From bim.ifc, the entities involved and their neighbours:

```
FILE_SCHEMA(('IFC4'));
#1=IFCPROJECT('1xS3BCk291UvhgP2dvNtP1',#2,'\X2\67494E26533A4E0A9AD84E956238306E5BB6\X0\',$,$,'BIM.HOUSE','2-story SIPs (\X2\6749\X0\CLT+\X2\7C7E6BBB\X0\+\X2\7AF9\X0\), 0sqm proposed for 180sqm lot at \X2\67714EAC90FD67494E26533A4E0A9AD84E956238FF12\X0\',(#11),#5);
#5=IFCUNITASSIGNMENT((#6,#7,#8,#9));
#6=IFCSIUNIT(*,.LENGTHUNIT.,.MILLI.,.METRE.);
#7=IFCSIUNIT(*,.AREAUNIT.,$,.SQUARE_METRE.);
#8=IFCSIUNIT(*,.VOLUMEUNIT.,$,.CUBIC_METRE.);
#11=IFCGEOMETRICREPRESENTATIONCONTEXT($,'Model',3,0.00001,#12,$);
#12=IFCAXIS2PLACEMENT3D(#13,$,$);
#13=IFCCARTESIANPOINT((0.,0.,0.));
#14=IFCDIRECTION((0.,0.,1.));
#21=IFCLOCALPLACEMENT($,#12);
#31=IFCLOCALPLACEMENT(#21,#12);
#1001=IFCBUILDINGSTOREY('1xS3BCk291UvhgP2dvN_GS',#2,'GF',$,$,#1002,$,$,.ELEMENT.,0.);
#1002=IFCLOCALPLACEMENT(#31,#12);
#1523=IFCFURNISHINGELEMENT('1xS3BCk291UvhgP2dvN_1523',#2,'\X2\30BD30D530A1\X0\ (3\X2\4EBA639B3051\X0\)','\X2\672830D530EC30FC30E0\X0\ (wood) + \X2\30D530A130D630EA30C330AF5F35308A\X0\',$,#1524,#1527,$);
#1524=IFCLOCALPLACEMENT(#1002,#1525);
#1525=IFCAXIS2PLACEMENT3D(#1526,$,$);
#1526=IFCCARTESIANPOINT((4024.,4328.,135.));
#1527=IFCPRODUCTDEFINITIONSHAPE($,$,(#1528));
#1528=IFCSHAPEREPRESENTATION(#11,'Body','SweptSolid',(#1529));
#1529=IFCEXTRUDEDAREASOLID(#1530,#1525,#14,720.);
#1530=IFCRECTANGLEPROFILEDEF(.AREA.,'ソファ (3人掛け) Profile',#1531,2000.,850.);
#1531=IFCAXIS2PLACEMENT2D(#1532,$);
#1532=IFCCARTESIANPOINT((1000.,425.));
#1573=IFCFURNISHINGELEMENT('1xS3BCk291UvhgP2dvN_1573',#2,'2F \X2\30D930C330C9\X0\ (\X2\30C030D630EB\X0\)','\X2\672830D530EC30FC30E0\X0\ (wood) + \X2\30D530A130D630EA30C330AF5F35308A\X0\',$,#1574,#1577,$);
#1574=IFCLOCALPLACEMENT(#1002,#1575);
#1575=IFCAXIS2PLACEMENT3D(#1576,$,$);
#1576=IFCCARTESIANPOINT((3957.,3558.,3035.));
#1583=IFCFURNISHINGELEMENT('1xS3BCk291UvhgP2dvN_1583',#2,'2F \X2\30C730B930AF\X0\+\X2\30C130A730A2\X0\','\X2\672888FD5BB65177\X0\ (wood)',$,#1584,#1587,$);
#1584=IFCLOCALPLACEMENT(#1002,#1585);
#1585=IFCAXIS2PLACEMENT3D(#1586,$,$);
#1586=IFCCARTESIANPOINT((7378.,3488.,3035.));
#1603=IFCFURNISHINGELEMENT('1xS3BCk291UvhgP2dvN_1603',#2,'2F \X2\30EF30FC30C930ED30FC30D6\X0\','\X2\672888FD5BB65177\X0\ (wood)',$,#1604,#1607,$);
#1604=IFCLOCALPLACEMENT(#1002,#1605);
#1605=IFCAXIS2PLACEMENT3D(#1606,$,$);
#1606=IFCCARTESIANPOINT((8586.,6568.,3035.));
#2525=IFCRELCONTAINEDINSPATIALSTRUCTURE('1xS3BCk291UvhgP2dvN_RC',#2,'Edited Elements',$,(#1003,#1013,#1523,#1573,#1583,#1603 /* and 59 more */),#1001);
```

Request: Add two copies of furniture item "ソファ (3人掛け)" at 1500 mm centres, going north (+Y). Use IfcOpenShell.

```python
import numpy as np
import ifcopenshell
import ifcopenshell.api.geometry
import ifcopenshell.api.root
import ifcopenshell.util.element
import ifcopenshell.util.placement
import ifcopenshell.util.unit

model = ifcopenshell.open("bim.ifc")
unit_scale = ifcopenshell.util.unit.calculate_unit_scale(model)


def reuse_history(source, copy):
    """copy_class also copies each property set's owner history, people and application; keep the originals."""
    for rel in copy.IsDefinedBy:
        if rel.is_a("IfcRelDefinesByProperties") and (history := rel.RelatingPropertyDefinition.OwnerHistory):
            rel.RelatingPropertyDefinition.OwnerHistory = source.OwnerHistory
            ifcopenshell.util.element.remove_deep2(model, history)


source = model.by_guid("1xS3BCk291UvhgP2dvN_1523")
base = ifcopenshell.util.placement.get_local_placement(source.ObjectPlacement)
step = np.array([0.0, 1.0, 0.0]) * 1.5 / unit_scale

for i in range(1, 3):
    copy = ifcopenshell.api.root.copy_class(model, product=source)
    copy.Representation = ifcopenshell.util.element.copy_deep(
        model, source.Representation, exclude=["IfcGeometricRepresentationContext", "IfcRepresentationMap"]
    )
    reuse_history(source, copy)
    matrix = base.copy()
    matrix[:3, 3] += i * step
    print("added at", matrix[:3, 3].round(3) + 0.0)
    ifcopenshell.api.geometry.edit_object_placement(model, product=copy, matrix=matrix, is_si=False)

model.write("bim_edited.ifc")
```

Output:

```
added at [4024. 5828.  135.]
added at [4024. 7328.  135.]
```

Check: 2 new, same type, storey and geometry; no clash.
